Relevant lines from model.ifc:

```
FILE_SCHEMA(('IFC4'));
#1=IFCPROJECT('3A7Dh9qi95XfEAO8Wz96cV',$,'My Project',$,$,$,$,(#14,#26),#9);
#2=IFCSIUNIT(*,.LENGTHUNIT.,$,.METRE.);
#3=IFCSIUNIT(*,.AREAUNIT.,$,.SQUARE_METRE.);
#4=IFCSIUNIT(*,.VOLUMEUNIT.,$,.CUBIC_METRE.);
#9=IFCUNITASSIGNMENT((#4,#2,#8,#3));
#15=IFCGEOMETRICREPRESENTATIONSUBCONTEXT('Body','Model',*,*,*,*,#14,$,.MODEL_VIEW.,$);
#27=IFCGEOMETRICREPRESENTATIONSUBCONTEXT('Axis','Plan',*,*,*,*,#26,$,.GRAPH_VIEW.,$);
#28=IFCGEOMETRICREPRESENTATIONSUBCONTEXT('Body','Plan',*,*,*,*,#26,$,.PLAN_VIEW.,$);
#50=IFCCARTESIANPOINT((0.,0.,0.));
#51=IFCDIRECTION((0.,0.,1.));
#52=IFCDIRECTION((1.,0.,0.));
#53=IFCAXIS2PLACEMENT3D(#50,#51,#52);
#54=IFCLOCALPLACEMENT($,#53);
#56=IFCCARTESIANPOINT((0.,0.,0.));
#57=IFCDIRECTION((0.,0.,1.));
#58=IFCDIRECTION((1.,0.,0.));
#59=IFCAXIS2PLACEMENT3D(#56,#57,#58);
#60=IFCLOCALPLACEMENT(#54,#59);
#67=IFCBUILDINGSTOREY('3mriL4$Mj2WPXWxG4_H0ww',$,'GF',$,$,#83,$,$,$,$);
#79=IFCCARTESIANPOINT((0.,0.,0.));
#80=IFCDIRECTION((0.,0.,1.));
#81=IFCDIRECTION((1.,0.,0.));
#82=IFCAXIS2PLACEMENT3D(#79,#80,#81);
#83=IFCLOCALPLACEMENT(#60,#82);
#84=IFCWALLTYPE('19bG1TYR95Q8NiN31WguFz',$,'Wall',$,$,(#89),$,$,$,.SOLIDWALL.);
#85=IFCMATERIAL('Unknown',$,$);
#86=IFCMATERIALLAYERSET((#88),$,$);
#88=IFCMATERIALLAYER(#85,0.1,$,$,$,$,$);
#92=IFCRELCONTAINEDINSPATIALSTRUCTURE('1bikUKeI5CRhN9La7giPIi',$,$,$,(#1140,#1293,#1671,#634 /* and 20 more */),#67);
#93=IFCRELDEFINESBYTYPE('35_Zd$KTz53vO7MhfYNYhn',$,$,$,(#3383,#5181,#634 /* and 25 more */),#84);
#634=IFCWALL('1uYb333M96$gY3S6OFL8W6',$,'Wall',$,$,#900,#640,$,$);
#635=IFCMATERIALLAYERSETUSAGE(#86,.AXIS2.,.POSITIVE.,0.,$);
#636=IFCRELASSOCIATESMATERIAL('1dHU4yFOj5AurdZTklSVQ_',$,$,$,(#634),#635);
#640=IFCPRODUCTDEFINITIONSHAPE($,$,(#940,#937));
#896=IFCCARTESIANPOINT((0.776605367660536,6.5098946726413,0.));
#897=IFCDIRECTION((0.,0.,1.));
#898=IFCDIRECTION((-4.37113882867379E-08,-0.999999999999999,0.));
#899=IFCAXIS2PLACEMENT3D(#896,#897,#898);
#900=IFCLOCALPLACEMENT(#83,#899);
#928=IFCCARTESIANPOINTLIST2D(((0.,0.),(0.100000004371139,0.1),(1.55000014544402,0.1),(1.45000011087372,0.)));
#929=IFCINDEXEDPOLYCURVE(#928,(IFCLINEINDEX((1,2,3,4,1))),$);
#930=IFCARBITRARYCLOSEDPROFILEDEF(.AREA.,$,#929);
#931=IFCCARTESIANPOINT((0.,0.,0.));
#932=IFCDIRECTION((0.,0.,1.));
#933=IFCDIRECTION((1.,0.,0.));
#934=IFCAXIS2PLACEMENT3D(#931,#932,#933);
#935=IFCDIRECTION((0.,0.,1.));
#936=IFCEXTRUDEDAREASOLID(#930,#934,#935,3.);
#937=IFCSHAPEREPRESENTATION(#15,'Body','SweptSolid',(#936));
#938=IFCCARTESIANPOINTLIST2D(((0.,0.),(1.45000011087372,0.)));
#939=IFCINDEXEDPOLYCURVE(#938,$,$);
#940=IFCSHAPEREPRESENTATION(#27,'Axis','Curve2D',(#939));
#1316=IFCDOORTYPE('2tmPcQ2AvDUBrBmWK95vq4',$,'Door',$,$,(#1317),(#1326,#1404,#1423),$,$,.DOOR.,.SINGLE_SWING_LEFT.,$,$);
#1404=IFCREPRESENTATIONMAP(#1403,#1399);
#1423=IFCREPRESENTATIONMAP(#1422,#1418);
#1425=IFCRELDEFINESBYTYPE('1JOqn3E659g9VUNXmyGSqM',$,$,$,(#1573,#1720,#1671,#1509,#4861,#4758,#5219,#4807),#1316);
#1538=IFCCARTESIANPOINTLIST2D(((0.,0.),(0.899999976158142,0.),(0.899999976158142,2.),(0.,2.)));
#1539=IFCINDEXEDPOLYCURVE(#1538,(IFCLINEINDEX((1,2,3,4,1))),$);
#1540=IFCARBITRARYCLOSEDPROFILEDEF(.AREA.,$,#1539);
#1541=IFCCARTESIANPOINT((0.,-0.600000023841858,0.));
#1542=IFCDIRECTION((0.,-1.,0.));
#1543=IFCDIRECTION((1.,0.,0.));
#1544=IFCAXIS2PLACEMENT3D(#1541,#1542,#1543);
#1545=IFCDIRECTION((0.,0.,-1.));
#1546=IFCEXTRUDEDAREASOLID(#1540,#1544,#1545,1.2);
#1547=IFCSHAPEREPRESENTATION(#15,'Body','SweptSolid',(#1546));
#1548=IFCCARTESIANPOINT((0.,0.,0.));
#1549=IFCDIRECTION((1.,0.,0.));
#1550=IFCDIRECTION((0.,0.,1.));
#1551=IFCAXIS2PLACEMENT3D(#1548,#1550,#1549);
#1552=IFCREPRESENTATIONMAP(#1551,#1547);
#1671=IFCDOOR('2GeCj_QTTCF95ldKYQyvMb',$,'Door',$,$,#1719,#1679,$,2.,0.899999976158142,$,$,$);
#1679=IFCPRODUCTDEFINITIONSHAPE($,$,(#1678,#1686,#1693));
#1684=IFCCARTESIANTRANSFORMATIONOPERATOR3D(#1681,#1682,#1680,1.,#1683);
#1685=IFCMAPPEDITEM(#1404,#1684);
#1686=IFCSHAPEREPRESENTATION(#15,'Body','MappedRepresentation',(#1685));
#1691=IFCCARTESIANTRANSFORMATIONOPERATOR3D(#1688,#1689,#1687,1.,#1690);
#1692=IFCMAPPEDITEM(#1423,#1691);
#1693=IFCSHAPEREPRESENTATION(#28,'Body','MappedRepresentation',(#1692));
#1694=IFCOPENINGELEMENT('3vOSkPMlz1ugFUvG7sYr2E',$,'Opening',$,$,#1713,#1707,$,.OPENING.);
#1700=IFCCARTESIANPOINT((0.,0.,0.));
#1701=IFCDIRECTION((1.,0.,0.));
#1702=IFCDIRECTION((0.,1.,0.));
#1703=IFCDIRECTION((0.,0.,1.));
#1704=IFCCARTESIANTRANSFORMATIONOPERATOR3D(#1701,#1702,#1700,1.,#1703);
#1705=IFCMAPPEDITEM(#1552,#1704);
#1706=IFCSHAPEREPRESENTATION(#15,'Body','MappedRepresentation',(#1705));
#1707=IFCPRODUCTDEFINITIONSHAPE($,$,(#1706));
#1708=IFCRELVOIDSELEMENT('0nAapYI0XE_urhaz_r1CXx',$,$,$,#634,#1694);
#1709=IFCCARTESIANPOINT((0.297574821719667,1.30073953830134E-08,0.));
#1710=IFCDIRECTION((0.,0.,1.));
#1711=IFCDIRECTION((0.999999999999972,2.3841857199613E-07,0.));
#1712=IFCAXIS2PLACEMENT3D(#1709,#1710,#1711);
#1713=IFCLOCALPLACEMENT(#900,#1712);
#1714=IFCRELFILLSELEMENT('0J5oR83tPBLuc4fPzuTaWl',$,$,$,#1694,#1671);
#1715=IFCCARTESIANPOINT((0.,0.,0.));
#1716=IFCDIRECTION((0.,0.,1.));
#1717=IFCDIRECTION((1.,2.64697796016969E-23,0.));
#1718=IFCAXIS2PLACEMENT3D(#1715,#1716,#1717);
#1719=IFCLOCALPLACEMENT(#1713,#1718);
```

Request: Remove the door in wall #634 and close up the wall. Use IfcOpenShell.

```python
import ifcopenshell
import ifcopenshell.api.feature
import ifcopenshell.api.root
import ifcopenshell.geom
import ifcopenshell.util.shape

model = ifcopenshell.open("model.ifc")
settings = ifcopenshell.geom.settings()


def volume(element):
    """Net volume in cubic metres, openings subtracted."""
    shape = ifcopenshell.geom.create_shape(settings, element)
    return ifcopenshell.util.shape.get_volume(shape.geometry)


door = model.by_guid("2GeCj_QTTCF95ldKYQyvMb")
opening = door.FillsVoids[0].RelatingOpeningElement
wall = opening.VoidsElements[0].RelatingBuildingElement
before = volume(wall)

ifcopenshell.api.root.remove_product(model, product=door)
ifcopenshell.api.feature.remove_feature(model, feature=opening)

after = volume(wall)

print(f"wall volume {before:.3f} -> {after:.3f} m3")

model.write("model_updated.ifc")
```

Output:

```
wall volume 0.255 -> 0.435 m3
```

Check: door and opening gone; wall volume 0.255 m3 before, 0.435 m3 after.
